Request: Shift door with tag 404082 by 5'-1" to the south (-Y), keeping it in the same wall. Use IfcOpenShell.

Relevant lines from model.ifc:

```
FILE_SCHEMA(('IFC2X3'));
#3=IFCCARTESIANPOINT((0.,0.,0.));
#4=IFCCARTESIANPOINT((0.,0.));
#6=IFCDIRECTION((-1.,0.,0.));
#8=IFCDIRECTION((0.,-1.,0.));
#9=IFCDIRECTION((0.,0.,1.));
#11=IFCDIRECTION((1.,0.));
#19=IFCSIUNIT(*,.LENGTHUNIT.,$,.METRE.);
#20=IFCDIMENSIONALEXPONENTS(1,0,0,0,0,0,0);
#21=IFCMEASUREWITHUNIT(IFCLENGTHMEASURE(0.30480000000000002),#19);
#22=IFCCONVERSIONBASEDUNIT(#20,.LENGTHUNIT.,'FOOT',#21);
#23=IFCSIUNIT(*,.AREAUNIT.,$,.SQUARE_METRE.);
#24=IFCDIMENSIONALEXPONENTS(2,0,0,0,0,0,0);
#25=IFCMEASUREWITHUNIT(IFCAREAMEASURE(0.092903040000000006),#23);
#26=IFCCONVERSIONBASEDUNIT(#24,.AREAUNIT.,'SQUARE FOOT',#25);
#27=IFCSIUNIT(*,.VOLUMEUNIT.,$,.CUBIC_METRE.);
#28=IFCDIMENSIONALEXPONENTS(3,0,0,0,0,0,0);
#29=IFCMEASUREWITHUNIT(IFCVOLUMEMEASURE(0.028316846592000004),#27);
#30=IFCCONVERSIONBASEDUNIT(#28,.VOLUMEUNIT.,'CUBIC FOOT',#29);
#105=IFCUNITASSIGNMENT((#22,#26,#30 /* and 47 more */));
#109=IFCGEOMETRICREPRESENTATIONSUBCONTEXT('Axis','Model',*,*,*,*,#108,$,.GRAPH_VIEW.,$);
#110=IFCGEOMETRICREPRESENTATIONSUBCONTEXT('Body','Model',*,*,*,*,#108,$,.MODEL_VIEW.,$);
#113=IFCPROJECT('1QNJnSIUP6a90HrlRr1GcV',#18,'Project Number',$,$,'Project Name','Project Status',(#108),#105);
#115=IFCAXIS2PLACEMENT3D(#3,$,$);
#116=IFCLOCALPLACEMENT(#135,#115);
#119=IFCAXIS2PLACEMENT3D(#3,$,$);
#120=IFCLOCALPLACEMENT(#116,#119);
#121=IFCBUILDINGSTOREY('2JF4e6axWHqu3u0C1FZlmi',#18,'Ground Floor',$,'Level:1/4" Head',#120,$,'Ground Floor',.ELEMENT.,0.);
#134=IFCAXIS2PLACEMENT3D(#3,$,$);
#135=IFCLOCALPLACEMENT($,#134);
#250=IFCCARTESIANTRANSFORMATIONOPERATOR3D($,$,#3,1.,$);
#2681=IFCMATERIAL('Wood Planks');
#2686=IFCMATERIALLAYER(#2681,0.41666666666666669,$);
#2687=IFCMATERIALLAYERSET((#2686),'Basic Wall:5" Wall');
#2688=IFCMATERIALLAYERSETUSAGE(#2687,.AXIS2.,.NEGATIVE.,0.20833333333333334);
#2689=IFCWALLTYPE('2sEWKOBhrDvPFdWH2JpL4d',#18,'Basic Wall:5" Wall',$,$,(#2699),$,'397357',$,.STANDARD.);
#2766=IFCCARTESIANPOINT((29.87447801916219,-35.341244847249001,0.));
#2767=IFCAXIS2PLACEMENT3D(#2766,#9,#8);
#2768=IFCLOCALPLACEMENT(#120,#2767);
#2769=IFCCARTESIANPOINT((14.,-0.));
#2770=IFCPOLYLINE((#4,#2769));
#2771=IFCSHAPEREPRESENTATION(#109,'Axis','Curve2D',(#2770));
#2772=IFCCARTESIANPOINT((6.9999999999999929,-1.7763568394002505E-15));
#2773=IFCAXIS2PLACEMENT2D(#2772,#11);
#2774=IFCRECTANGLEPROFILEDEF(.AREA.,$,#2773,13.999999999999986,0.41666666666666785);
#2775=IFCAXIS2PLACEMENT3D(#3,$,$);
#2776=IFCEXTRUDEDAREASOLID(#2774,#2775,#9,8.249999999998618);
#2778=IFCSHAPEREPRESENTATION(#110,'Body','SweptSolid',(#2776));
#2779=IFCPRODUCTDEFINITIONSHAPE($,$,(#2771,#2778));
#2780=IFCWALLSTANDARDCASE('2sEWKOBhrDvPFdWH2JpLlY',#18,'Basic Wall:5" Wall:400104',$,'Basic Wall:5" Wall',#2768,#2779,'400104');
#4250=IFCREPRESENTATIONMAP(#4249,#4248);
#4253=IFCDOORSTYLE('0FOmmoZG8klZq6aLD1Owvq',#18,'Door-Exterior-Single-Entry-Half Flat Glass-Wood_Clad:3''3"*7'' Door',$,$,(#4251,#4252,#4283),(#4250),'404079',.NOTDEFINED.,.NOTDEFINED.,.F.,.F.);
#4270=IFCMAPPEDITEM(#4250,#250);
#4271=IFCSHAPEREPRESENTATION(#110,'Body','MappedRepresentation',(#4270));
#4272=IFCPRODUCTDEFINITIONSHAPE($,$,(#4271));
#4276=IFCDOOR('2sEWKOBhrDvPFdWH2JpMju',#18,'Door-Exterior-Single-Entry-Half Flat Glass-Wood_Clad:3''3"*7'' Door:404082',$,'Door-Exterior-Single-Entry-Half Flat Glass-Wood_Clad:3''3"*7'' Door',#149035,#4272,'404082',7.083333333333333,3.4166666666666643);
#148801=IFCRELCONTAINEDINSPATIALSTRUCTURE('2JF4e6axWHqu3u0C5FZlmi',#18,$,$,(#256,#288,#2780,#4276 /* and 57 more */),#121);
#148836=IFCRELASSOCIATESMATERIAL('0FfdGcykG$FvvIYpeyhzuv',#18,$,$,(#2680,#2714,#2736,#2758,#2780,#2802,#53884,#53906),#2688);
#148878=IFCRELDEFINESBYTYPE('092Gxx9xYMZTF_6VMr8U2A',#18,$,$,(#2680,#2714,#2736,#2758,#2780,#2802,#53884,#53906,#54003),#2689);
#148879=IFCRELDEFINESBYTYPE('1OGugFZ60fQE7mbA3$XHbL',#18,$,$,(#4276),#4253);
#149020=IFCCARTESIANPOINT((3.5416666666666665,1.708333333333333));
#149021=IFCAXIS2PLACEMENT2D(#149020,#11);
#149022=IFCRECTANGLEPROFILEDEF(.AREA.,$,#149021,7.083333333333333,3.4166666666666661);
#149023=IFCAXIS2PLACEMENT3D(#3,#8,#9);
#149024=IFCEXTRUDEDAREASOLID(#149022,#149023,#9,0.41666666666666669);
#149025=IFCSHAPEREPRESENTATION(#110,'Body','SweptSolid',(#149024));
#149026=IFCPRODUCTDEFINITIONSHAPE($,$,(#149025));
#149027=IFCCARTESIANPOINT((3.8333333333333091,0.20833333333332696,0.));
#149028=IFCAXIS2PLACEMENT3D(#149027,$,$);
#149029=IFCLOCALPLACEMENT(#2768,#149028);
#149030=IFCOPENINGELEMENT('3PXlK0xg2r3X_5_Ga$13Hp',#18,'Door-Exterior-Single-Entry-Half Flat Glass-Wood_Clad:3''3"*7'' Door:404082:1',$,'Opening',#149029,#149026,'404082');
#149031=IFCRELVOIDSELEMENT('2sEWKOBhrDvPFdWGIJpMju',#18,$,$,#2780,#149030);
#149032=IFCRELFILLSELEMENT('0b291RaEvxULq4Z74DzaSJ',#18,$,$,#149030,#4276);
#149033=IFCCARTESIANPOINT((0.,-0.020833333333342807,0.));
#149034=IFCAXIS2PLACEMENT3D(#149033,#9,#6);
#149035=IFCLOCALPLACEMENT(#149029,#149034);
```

```python
import ifcopenshell
import ifcopenshell.api.geometry
import ifcopenshell.util.placement
import ifcopenshell.util.unit

model = ifcopenshell.open("model.ifc")
unit_scale = ifcopenshell.util.unit.calculate_unit_scale(model)

door = model.by_id(4276)
opening = door.FillsVoids[0].RelatingOpeningElement
wall = opening.VoidsElements[0].RelatingBuildingElement

wall_matrix = ifcopenshell.util.placement.get_local_placement(wall.ObjectPlacement)
shift = wall_matrix[:3, 0] * 61 * 0.0254 / unit_scale
before = ifcopenshell.util.placement.get_local_placement(door.ObjectPlacement)[:3, 3].copy()

# The door is placed relative to its opening, so it follows when the opening moves.
matrix = ifcopenshell.util.placement.get_local_placement(opening.ObjectPlacement)
matrix[:3, 3] += shift
ifcopenshell.api.geometry.edit_object_placement(
    model, product=opening, matrix=matrix, is_si=False, should_transform_children=True
)

after = ifcopenshell.util.placement.get_local_placement(door.ObjectPlacement)[:3, 3]
print("door moved by", (after - before).round(3) + 0.0)

model.write("model-out.ifc")
```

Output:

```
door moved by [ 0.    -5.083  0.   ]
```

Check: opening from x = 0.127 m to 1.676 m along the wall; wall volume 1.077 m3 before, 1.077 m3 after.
